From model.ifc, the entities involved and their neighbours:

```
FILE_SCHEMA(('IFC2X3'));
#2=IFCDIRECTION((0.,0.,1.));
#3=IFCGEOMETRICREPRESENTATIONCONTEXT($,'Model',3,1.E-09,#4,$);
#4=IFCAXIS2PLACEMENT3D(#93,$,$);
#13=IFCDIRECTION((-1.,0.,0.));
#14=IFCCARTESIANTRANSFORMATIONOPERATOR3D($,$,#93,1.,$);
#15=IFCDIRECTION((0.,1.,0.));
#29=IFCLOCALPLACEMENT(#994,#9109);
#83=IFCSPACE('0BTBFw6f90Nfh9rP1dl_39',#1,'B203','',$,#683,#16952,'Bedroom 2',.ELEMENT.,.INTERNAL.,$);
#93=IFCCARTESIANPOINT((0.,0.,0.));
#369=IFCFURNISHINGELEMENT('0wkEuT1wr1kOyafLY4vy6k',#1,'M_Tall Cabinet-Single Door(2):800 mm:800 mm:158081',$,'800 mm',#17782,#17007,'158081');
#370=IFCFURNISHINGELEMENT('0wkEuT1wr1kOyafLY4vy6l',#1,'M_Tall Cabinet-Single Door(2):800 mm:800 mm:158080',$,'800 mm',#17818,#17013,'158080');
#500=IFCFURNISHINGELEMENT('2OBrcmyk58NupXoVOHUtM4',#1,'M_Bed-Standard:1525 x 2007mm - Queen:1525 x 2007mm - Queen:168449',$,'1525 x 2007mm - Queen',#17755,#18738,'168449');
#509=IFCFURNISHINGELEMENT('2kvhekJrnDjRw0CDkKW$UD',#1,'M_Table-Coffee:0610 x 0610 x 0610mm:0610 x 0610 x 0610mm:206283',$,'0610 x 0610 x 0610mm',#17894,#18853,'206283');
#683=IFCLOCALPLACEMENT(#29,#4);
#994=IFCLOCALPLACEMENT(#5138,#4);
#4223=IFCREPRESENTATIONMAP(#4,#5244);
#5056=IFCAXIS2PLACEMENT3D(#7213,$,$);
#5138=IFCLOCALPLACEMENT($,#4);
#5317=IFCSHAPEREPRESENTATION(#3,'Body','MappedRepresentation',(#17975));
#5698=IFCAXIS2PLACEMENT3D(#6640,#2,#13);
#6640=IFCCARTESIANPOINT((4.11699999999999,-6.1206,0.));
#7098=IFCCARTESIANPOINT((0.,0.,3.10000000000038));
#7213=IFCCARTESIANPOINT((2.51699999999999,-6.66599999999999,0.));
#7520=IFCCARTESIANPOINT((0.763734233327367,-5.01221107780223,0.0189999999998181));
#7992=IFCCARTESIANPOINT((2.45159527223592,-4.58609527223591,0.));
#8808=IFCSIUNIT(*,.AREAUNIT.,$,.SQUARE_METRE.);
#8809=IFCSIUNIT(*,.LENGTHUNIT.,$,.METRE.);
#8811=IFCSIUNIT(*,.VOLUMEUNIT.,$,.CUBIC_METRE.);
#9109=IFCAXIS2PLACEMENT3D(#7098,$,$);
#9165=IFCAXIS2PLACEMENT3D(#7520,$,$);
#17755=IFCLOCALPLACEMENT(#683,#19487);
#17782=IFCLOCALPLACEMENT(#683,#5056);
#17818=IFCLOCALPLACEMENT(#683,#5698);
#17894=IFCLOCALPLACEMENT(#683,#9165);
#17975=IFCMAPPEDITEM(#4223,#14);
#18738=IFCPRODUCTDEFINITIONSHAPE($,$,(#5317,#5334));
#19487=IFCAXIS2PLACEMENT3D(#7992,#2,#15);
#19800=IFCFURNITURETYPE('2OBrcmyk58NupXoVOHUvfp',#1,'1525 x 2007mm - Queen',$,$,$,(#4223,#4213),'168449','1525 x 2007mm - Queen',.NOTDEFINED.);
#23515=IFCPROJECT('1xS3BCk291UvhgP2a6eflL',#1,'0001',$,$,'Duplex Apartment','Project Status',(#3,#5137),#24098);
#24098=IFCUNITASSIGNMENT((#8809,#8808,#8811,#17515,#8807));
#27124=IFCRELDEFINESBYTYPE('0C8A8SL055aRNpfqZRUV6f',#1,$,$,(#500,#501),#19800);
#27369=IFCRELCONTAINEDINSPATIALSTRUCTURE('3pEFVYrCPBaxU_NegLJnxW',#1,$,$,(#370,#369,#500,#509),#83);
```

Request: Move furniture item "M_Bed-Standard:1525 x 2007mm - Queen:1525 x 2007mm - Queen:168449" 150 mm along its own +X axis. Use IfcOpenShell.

```python
import ifcopenshell
import ifcopenshell.api.geometry
import ifcopenshell.util.placement
import ifcopenshell.util.unit

model = ifcopenshell.open("model.ifc")
unit_scale = ifcopenshell.util.unit.calculate_unit_scale(model)

item = model.by_guid("2OBrcmyk58NupXoVOHUtM4")
matrix = ifcopenshell.util.placement.get_local_placement(item.ObjectPlacement)
matrix[:3, 3] += matrix[:3, 0] * 0.15 / unit_scale
ifcopenshell.api.geometry.edit_object_placement(model, product=item, matrix=matrix, is_si=False)

print(ifcopenshell.util.placement.get_local_placement(item.ObjectPlacement).round(3) + 0.0)

model.write("model-out.ifc")
```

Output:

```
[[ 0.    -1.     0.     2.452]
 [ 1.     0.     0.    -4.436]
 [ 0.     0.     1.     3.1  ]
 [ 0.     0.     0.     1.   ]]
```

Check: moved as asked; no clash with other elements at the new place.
